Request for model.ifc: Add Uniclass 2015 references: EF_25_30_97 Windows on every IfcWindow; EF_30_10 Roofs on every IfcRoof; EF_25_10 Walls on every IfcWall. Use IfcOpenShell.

First a look at what the model holds.

```python
import ifcopenshell

model = ifcopenshell.open("model.ifc")
print(model.schema)
print("classifications:", [c.Name for c in model.by_type("IfcClassification")])
for ifc_class in ("IfcDoor", "IfcRoof", "IfcStair", "IfcWall", "IfcWindow"):
    print(ifc_class, len(model.by_type(ifc_class)))
```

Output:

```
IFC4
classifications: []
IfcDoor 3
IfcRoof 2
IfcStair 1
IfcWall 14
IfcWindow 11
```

```python
import ifcopenshell
import ifcopenshell.api.classification

model = ifcopenshell.open("model.ifc")

system = ifcopenshell.api.classification.add_classification(model, classification="Uniclass 2015")

codes = {
    "IfcWindow": ("EF_25_30_97", "Windows"),
    "IfcRoof": ("EF_30_10", "Roofs"),
    "IfcWall": ("EF_25_10", "Walls"),
}
for ifc_class, (code, name) in codes.items():
    products = model.by_type(ifc_class)
    ifcopenshell.api.classification.add_reference(
        model, products=products, classification=system, identification=code, name=name
    )
    print(code, len(products))

model.write("model_updated.ifc")
```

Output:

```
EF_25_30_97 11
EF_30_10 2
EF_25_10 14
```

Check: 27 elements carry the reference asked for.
